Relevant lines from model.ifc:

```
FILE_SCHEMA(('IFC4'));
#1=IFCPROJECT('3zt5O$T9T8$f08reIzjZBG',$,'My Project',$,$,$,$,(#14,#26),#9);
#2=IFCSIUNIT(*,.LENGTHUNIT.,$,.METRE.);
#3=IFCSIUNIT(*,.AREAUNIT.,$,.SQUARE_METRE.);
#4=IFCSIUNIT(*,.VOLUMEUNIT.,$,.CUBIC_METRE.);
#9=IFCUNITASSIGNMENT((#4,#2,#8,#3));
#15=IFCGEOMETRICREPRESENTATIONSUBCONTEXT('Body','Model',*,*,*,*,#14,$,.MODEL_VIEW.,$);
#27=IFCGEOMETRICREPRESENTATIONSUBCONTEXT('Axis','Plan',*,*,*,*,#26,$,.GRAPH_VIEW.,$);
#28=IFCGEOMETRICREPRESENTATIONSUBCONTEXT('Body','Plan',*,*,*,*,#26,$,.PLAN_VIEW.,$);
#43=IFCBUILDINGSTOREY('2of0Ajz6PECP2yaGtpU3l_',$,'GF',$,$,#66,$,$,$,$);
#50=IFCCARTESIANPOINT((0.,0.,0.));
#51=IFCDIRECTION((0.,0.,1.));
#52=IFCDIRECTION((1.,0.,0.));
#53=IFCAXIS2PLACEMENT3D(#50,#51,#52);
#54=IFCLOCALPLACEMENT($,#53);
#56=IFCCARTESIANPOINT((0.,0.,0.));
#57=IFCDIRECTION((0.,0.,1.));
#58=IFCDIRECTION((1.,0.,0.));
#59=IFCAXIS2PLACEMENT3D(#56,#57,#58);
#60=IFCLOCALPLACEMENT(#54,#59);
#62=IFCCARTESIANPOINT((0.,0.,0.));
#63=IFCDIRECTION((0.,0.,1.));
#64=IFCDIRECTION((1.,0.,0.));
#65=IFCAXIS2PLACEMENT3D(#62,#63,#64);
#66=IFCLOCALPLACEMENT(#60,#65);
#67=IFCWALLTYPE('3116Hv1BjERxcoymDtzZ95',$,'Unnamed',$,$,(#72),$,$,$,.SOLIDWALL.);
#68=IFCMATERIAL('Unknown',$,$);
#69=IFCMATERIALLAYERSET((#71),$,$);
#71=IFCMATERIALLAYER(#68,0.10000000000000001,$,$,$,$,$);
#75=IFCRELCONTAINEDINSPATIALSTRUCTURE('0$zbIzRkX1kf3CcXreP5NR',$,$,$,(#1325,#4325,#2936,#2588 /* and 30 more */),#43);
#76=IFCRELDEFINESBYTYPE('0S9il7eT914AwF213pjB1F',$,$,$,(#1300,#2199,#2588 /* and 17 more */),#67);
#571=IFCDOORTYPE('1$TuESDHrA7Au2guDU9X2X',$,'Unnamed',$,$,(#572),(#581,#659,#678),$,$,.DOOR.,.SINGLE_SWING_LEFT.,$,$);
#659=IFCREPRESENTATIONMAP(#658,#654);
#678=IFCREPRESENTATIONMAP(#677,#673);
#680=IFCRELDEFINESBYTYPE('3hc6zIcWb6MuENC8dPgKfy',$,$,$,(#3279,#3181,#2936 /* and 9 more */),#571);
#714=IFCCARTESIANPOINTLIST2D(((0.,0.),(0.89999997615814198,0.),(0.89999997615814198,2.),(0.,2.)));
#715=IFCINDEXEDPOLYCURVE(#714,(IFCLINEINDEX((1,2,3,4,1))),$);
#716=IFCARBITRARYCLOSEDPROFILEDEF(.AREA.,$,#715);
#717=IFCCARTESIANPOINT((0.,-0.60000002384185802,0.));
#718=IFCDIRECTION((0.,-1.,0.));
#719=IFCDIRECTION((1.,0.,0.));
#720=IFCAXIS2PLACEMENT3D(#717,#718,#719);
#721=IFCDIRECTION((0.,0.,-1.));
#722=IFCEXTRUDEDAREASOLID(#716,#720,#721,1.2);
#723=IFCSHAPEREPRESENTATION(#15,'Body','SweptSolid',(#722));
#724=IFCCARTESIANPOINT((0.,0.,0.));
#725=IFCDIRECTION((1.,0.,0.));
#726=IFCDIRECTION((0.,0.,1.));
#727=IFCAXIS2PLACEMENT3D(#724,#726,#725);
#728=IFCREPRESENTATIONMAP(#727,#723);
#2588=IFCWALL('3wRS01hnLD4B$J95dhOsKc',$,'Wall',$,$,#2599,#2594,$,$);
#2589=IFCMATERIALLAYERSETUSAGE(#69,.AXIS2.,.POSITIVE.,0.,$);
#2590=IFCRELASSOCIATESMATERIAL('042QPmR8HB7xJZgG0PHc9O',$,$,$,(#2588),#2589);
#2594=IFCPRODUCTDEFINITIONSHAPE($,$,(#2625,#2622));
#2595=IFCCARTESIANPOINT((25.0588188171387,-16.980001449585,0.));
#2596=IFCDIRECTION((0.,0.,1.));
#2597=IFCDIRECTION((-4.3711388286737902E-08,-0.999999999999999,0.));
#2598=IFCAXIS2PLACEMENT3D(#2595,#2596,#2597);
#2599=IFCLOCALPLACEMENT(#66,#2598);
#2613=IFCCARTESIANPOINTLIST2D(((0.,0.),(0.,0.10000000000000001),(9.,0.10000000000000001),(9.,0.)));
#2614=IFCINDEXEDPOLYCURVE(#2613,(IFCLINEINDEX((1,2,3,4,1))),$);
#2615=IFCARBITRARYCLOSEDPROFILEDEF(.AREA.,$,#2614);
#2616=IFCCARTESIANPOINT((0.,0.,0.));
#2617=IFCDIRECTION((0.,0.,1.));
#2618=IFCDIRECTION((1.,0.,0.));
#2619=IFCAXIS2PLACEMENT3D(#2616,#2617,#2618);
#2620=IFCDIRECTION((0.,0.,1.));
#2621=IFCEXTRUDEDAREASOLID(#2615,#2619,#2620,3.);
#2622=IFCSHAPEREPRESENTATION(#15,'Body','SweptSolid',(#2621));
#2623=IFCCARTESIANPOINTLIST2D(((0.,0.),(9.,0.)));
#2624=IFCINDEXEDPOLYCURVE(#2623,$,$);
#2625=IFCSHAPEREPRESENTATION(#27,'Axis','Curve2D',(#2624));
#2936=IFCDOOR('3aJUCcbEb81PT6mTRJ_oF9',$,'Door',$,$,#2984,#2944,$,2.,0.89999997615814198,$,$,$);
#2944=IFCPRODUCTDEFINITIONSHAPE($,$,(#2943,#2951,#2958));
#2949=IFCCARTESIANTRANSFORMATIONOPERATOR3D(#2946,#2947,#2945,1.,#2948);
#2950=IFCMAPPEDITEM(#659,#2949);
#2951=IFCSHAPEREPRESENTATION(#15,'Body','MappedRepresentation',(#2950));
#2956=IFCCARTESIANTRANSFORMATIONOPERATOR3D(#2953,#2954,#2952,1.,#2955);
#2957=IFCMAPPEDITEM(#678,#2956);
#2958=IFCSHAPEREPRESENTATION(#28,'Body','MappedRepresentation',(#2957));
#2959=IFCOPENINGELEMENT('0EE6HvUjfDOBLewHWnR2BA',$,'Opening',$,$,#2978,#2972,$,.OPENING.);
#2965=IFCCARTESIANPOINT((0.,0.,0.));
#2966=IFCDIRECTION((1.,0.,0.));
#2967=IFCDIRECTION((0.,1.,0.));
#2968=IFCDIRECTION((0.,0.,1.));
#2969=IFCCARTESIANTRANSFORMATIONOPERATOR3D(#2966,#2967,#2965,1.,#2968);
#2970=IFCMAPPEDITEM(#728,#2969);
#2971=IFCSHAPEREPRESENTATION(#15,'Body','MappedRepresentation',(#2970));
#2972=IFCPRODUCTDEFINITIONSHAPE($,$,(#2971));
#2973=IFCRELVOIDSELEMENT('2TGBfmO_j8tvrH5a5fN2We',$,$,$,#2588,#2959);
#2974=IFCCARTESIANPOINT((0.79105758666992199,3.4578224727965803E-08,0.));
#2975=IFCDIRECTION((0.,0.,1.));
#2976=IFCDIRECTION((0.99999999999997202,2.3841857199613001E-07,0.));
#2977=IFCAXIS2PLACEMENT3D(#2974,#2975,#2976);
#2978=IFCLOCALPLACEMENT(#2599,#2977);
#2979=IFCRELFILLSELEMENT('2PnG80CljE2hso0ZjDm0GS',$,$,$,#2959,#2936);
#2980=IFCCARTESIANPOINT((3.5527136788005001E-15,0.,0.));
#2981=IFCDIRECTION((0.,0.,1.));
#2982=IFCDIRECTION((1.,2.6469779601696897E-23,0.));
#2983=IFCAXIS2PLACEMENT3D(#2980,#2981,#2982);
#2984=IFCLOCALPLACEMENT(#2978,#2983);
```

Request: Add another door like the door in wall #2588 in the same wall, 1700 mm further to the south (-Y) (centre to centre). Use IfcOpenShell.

```python
import ifcopenshell
import ifcopenshell.api.feature
import ifcopenshell.api.geometry
import ifcopenshell.api.root
import ifcopenshell.geom
import ifcopenshell.util.element
import ifcopenshell.util.placement
import ifcopenshell.util.shape
import ifcopenshell.util.unit

model = ifcopenshell.open("model.ifc")
unit_scale = ifcopenshell.util.unit.calculate_unit_scale(model)
settings = ifcopenshell.geom.settings()


def volume(element):
    """Net volume in cubic metres, openings subtracted."""
    shape = ifcopenshell.geom.create_shape(settings, element)
    return ifcopenshell.util.shape.get_volume(shape.geometry)


door = model.by_guid("3aJUCcbEb81PT6mTRJ_oF9")
opening = door.FillsVoids[0].RelatingOpeningElement
wall = opening.VoidsElements[0].RelatingBuildingElement
before = volume(wall)
shift = ifcopenshell.util.placement.get_local_placement(wall.ObjectPlacement)[:3, 0] * 1.7 / unit_scale

# copy_class copies the void relationship, type, container and properties, but no geometry.
new_opening = ifcopenshell.api.root.copy_class(model, product=opening)
new_opening.Representation = ifcopenshell.util.element.copy_deep(
    model, opening.Representation, exclude=["IfcGeometricRepresentationContext", "IfcRepresentationMap"]
)
new_door = ifcopenshell.api.root.copy_class(model, product=door)
new_door.Representation = ifcopenshell.util.element.copy_deep(
    model, door.Representation, exclude=["IfcGeometricRepresentationContext", "IfcRepresentationMap"]
)
ifcopenshell.api.feature.add_filling(model, opening=new_opening, element=new_door)

for old, new in ((opening, new_opening), (door, new_door)):
    matrix = ifcopenshell.util.placement.get_local_placement(old.ObjectPlacement)
    matrix[:3, 3] += shift
    ifcopenshell.api.geometry.edit_object_placement(model, product=new, matrix=matrix, is_si=False)

after = volume(wall)

print(f"wall volume {before:.3f} -> {after:.3f} m3")

model.write("model_edited.ifc")
```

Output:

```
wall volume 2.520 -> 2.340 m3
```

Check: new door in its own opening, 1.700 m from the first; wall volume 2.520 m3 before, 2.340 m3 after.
